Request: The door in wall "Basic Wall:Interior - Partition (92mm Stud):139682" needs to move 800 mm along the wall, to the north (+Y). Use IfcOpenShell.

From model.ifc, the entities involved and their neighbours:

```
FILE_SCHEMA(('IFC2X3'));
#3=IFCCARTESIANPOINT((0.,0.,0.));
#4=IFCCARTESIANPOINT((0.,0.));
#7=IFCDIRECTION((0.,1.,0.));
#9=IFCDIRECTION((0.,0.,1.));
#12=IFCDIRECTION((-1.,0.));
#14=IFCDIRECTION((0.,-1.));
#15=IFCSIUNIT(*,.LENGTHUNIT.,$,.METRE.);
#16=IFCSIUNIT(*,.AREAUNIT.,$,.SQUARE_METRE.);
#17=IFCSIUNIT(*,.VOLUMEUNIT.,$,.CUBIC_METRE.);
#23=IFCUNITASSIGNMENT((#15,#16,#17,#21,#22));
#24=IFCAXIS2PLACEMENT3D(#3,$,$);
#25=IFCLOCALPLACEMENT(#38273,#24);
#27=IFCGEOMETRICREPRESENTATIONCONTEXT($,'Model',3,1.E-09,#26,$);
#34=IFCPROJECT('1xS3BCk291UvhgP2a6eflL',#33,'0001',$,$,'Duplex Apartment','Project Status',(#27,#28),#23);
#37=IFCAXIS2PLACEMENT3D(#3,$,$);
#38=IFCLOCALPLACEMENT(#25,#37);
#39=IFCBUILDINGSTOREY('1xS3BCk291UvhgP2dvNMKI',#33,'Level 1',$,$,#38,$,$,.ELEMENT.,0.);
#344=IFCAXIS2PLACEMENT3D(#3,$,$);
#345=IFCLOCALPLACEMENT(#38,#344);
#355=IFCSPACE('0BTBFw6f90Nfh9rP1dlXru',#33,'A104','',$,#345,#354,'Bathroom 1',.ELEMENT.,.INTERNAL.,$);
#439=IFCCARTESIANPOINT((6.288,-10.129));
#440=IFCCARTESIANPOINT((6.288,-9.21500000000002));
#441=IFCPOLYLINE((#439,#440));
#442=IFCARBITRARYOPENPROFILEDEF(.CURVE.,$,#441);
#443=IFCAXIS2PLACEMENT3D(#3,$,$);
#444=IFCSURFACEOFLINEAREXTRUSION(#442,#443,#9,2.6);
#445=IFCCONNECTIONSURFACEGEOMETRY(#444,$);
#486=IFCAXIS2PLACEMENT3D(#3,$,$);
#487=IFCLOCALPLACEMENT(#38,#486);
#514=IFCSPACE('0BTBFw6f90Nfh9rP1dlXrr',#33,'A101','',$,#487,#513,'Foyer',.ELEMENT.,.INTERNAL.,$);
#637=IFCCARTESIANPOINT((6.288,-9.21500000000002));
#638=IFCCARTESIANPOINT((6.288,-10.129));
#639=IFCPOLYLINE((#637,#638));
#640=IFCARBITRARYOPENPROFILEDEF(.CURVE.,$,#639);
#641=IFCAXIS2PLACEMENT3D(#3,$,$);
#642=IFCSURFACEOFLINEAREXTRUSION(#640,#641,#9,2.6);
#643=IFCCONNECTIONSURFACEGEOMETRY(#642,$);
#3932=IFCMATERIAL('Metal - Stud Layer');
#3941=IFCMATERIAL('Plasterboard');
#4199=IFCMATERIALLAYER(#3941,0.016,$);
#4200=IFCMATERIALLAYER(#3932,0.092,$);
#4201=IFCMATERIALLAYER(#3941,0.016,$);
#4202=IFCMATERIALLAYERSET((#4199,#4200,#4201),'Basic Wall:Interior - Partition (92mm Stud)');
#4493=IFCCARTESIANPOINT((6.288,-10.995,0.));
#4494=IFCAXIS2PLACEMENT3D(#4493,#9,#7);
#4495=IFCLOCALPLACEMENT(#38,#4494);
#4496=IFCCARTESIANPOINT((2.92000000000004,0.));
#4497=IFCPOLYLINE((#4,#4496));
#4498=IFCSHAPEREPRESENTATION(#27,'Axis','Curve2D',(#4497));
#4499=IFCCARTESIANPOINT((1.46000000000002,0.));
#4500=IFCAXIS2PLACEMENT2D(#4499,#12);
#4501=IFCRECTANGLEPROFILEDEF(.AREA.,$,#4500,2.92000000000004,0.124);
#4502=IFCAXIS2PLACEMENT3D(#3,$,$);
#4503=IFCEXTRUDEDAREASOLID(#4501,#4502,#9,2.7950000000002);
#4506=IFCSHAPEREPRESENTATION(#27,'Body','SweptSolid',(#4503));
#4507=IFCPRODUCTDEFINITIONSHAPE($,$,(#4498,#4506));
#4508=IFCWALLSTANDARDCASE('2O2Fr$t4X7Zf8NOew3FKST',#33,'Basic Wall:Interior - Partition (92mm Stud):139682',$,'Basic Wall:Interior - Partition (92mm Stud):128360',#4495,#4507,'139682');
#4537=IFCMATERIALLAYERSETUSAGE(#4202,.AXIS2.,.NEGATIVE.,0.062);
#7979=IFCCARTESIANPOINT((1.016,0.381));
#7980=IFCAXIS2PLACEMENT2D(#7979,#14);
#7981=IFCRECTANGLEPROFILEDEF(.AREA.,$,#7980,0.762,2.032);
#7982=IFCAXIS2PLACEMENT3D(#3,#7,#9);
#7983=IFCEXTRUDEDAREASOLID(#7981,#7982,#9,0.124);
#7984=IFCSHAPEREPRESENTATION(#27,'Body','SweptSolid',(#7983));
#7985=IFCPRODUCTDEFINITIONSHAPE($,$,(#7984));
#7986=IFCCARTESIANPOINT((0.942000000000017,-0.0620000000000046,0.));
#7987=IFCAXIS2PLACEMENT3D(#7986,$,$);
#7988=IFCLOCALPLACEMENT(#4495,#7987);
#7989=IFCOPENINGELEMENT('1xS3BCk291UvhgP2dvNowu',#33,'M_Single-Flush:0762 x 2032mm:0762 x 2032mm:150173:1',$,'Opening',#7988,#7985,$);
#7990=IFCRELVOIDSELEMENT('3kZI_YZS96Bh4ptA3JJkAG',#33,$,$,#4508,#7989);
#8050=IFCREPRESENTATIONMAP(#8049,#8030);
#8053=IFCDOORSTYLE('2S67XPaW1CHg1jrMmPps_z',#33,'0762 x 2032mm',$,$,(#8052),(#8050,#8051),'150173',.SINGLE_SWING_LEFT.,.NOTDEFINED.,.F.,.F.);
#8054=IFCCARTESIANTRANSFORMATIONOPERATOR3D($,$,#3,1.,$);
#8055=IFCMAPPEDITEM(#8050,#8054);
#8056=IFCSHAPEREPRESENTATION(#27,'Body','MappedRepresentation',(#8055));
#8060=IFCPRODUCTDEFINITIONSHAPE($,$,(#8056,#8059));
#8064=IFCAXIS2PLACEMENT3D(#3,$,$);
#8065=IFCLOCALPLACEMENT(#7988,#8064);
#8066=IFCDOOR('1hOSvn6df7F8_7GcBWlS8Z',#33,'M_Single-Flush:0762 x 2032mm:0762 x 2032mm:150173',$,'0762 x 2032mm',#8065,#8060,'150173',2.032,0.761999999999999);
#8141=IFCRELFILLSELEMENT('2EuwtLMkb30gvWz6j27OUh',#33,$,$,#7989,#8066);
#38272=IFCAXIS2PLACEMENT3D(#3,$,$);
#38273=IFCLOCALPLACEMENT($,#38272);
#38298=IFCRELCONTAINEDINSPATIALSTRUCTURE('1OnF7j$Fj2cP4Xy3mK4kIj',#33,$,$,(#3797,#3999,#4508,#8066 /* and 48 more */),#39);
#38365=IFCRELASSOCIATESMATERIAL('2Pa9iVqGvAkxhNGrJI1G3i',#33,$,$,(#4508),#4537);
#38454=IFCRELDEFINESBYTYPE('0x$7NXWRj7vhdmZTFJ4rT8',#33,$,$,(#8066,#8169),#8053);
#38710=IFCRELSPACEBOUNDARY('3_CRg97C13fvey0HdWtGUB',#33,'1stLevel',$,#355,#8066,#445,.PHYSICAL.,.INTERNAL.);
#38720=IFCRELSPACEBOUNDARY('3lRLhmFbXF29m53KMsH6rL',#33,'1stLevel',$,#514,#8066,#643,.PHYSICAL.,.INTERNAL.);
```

```python
import numpy as np
import ifcopenshell
import ifcopenshell.api.geometry
import ifcopenshell.util.placement
import ifcopenshell.util.unit

model = ifcopenshell.open("model.ifc")
unit_scale = ifcopenshell.util.unit.calculate_unit_scale(model)

door = model.by_guid("1hOSvn6df7F8_7GcBWlS8Z")
opening = door.FillsVoids[0].RelatingOpeningElement
wall = opening.VoidsElements[0].RelatingBuildingElement

wall_matrix = ifcopenshell.util.placement.get_local_placement(wall.ObjectPlacement)
shift = wall_matrix[:3, 0] * 0.8 / unit_scale
before = ifcopenshell.util.placement.get_local_placement(door.ObjectPlacement)[:3, 3].copy()

# The door is placed relative to its opening, so it follows when the opening moves.
matrix = ifcopenshell.util.placement.get_local_placement(opening.ObjectPlacement)
matrix[:3, 3] += shift
ifcopenshell.api.geometry.edit_object_placement(
    model, product=opening, matrix=matrix, is_si=False, should_transform_children=True
)

# Space boundary surfaces are stored in each space's coordinates; move them too.
for rel in door.ProvidesBoundaries:
    if not rel.ConnectionGeometry:
        continue
    surface = rel.ConnectionGeometry.SurfaceOnRelatingElement
    space_matrix = ifcopenshell.util.placement.get_local_placement(rel.RelatingSpace.ObjectPlacement)
    point = np.array(surface.Position.Location.Coordinates) + space_matrix[:3, :3].T @ shift
    surface.Position = model.createIfcAxis2Placement3D(
        model.createIfcCartesianPoint(point.tolist()), surface.Position.Axis, surface.Position.RefDirection
    )

after = ifcopenshell.util.placement.get_local_placement(door.ObjectPlacement)[:3, 3]
print("door moved by", (after - before).round(3) + 0.0)

model.write("model_updated.ifc")
```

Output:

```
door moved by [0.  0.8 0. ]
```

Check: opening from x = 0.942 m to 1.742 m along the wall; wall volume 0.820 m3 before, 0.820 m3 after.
